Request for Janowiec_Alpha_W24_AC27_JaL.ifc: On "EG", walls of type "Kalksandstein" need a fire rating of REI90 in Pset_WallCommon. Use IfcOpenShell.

First a look at what the model holds.

```python
import ifcopenshell
import ifcopenshell.util.element

model = ifcopenshell.open("Janowiec_Alpha_W24_AC27_JaL.ifc")
print(model.schema)
storey = next(s for s in model.by_type("IfcBuildingStorey") if s.Name == "EG")
walls = [e for e in ifcopenshell.util.element.get_decomposition(storey) if e.is_a("IfcWall")]
seen = {}
for e in walls:
    element_type = ifcopenshell.util.element.get_type(e)
    key = (element_type.Name if element_type != e and element_type else None, ifcopenshell.util.element.get_pset(e, "Pset_WallCommon", "FireRating"))
    seen[key] = seen.get(key, 0) + 1
for (name, value), count in sorted(seen.items(), key=str):
    print(count, "x", name, "|", value)
```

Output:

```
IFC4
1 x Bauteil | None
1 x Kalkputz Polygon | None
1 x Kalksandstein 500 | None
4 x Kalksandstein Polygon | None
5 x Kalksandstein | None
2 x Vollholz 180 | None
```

```python
import ifcopenshell
import ifcopenshell.api.pset
import ifcopenshell.util.element

model = ifcopenshell.open("Janowiec_Alpha_W24_AC27_JaL.ifc")

storey = next(s for s in model.by_type("IfcBuildingStorey") if s.Name == "EG")
walls = [e for e in ifcopenshell.util.element.get_decomposition(storey) if e.is_a("IfcWall")]

count = 0
for e in walls:
    element_type = ifcopenshell.util.element.get_type(e)
    if element_type in (None, e) or element_type.Name != "Kalksandstein":
        continue
    # add_pset returns the element's existing set when there is one.
    pset = ifcopenshell.api.pset.add_pset(model, product=e, name="Pset_WallCommon")
    ifcopenshell.api.pset.edit_pset(model, pset=pset, properties={"FireRating": "REI90"})
    count += 1

print(count, "walls updated")

model.write("Janowiec_Alpha_W24_AC27_JaL_edited.ifc")
```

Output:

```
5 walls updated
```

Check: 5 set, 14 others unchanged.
